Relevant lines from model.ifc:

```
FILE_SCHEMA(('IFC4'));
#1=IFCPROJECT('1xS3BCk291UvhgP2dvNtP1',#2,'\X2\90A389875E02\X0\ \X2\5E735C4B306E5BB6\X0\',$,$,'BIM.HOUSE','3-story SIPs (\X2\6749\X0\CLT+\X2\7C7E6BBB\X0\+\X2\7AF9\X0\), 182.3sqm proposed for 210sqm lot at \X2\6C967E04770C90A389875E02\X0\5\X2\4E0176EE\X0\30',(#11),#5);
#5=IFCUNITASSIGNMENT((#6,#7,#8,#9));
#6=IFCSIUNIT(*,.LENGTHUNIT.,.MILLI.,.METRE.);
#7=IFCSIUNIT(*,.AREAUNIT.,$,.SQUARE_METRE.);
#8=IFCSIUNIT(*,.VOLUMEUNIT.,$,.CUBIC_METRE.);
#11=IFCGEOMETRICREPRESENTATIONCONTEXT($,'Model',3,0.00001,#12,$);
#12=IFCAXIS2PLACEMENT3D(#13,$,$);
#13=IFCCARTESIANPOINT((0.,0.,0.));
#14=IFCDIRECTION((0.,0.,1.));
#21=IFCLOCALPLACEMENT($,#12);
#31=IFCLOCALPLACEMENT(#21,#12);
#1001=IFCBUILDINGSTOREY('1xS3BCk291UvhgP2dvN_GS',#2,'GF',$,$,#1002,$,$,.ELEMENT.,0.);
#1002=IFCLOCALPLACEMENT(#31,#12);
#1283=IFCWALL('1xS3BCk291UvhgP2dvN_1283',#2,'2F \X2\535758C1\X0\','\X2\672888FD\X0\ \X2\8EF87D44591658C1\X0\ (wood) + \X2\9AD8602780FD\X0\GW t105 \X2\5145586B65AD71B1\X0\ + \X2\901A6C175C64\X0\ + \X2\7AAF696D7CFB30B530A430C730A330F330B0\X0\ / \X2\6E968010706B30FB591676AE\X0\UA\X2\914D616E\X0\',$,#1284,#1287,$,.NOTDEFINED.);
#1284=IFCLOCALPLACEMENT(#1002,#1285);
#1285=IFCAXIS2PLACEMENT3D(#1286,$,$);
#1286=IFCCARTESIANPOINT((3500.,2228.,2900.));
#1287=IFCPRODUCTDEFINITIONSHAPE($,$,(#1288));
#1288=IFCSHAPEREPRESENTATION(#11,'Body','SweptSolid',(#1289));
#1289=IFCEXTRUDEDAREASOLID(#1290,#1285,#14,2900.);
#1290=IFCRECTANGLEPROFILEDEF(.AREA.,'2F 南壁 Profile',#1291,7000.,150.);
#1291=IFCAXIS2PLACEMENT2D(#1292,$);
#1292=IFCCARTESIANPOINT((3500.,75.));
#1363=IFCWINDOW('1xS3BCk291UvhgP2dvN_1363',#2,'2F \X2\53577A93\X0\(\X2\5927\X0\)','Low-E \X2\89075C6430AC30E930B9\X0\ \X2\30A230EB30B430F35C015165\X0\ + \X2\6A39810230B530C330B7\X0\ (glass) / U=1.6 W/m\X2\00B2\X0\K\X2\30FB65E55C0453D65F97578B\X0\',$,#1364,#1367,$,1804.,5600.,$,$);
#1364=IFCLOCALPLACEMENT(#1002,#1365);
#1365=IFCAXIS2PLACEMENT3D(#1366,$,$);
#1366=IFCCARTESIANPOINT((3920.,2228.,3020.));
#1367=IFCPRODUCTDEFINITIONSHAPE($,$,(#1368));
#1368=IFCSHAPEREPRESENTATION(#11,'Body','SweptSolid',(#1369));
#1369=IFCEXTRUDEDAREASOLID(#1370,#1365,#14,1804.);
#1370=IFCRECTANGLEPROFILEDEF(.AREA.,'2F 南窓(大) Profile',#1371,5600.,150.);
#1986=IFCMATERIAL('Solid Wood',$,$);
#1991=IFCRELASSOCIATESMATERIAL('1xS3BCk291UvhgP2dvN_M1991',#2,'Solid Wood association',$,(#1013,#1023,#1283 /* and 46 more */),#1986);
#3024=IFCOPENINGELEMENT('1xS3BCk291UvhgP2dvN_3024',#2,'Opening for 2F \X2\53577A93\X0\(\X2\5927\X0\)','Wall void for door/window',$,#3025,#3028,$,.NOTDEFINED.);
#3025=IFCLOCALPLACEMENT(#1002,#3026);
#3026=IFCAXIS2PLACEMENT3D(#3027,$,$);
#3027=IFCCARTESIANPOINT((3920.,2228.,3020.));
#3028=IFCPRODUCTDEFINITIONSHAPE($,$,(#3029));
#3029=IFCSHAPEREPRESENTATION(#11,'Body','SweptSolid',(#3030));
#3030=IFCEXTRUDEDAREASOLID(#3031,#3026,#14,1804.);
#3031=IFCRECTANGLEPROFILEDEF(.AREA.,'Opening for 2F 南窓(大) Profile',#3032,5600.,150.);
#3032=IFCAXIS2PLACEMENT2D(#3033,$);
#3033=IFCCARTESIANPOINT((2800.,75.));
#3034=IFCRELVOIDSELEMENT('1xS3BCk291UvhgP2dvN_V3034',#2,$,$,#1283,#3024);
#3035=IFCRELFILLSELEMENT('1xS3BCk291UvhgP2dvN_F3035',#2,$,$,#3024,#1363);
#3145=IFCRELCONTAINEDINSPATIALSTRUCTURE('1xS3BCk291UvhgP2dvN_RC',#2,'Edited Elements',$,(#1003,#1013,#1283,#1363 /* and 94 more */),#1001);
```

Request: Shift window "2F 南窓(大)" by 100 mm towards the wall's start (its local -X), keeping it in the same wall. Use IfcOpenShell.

```python
import ifcopenshell
import ifcopenshell.api.geometry
import ifcopenshell.util.placement
import ifcopenshell.util.unit

model = ifcopenshell.open("model.ifc")
unit_scale = ifcopenshell.util.unit.calculate_unit_scale(model)

window = model.by_guid("1xS3BCk291UvhgP2dvN_1363")
opening = window.FillsVoids[0].RelatingOpeningElement
wall = opening.VoidsElements[0].RelatingBuildingElement

wall_matrix = ifcopenshell.util.placement.get_local_placement(wall.ObjectPlacement)
shift = wall_matrix[:3, 0] * -0.1 / unit_scale
before = ifcopenshell.util.placement.get_local_placement(window.ObjectPlacement)[:3, 3].copy()

# The window is not placed relative to its opening, so move both.
for product in (opening, window):
    matrix = ifcopenshell.util.placement.get_local_placement(product.ObjectPlacement)
    matrix[:3, 3] += shift
    ifcopenshell.api.geometry.edit_object_placement(model, product=product, matrix=matrix, is_si=False)

after = ifcopenshell.util.placement.get_local_placement(window.ObjectPlacement)[:3, 3]
print("window moved by", (after - before).round(3) + 0.0)

model.write("model_rev.ifc")
```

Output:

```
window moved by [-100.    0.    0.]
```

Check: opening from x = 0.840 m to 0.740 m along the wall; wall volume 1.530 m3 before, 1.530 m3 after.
